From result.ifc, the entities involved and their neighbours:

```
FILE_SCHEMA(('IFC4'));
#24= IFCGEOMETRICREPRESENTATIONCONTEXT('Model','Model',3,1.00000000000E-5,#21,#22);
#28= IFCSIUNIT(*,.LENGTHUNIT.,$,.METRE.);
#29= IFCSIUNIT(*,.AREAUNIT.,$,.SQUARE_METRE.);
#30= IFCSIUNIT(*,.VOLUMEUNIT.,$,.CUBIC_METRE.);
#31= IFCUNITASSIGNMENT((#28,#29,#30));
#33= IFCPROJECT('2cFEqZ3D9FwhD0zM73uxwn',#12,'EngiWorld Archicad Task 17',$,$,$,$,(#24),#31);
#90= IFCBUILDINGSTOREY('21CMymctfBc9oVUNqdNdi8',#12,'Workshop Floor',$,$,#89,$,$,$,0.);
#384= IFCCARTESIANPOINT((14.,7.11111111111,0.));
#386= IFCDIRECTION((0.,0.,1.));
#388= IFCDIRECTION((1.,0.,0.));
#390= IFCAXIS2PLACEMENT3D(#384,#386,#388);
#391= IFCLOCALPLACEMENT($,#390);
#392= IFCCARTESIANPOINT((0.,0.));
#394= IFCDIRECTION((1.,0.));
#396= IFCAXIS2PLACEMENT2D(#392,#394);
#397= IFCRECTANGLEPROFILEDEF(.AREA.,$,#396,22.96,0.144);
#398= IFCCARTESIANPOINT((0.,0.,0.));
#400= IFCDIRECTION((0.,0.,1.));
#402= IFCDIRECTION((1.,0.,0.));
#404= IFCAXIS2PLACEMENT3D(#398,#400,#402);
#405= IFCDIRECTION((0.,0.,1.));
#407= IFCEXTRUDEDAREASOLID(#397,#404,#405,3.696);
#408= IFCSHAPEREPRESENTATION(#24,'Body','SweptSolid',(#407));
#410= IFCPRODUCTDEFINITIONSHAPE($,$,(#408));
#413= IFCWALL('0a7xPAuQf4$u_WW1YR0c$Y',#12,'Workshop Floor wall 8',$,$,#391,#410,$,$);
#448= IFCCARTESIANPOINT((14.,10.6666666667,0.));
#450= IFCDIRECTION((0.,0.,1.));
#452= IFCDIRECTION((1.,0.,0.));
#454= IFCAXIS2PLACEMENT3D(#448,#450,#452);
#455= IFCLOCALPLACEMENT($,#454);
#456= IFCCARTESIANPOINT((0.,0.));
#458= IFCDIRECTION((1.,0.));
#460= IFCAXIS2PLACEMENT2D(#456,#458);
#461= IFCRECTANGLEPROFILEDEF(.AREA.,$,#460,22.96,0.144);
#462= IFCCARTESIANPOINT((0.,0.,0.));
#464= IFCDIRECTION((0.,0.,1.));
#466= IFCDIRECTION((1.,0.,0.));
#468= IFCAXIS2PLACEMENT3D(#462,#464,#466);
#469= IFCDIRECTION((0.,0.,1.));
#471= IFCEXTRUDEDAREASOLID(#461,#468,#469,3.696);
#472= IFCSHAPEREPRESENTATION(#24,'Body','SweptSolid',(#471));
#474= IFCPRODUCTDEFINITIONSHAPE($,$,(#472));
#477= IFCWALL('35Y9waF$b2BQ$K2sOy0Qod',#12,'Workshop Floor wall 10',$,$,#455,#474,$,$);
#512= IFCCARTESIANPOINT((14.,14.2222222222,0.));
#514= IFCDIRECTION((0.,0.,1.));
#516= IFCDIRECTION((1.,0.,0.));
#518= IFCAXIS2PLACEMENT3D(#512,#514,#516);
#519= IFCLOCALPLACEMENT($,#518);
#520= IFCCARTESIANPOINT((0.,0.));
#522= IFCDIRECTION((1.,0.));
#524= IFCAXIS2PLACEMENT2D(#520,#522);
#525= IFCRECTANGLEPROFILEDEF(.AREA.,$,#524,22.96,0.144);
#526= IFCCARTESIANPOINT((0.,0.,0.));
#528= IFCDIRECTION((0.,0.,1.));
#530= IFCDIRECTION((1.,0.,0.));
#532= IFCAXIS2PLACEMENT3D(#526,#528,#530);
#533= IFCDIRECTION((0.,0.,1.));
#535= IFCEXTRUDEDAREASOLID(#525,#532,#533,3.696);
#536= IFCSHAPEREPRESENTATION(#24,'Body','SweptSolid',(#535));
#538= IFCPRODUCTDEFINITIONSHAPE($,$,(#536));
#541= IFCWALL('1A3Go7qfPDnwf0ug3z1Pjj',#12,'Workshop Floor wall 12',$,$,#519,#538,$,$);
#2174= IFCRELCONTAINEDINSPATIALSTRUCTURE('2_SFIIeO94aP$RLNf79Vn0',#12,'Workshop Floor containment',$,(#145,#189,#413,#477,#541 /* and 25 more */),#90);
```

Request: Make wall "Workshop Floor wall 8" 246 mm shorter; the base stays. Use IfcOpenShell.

```python
import ifcopenshell
import ifcopenshell.geom
import ifcopenshell.util.shape
import ifcopenshell.util.unit

model = ifcopenshell.open("result.ifc")
unit_scale = ifcopenshell.util.unit.calculate_unit_scale(model)
settings = ifcopenshell.geom.settings()


def volume(element):
    """Net volume in cubic metres, openings subtracted."""
    shape = ifcopenshell.geom.create_shape(settings, element)
    return ifcopenshell.util.shape.get_volume(shape.geometry)


wall = model.by_guid("0a7xPAuQf4$u_WW1YR0c$Y")
before = volume(wall)

body = next(r for r in wall.Representation.Representations if r.RepresentationIdentifier == "Body")
solid = body.Items[0]
old_height = solid.Depth
solid.Depth -= 0.246 / unit_scale
after = volume(wall)

print(f"height {old_height:g} -> {solid.Depth:g}, volume {before:.3f} -> {after:.3f} m3")

model.write("result_rev.ifc")
```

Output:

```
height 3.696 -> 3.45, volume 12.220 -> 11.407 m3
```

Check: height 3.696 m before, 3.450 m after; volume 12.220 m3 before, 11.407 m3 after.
